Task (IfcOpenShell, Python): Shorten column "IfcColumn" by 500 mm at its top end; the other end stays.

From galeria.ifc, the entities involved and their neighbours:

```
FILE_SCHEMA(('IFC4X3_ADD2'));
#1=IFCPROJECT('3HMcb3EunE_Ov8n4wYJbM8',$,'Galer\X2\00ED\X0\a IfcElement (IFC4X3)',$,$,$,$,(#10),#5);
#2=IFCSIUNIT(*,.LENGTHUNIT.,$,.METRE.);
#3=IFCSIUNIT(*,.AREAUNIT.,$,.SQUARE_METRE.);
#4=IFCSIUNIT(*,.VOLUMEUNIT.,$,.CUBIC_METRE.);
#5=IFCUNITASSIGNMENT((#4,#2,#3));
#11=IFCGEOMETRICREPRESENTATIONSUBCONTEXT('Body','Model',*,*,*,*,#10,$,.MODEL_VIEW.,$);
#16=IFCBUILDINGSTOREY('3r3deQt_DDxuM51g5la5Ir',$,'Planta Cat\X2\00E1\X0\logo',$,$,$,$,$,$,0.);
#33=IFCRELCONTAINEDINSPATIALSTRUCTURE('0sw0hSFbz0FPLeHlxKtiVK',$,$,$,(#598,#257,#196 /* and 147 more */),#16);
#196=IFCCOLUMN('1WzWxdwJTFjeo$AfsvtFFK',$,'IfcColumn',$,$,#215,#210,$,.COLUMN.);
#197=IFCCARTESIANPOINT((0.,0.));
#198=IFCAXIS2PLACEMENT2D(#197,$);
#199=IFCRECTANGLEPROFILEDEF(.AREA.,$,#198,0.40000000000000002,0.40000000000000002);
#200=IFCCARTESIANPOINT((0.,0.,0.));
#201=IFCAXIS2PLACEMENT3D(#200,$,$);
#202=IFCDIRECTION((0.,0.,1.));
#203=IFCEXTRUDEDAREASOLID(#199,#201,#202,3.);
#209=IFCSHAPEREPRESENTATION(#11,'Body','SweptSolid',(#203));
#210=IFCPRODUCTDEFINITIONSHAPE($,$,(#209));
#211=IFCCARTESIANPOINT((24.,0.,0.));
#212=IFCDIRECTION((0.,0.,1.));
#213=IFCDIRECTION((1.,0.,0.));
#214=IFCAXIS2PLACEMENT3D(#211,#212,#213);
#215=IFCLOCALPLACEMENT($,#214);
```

```python
import ifcopenshell
import ifcopenshell.util.representation
import ifcopenshell.util.unit

model = ifcopenshell.open("galeria.ifc")
unit_scale = ifcopenshell.util.unit.calculate_unit_scale(model)

member = model.by_id(196)
change = -0.5 / unit_scale

# The extrusion runs towards the end named, so only its depth changes.
body = ifcopenshell.util.representation.get_representation(member, "Model", "Body")
solid = body.Items[0]
old_length = solid.Depth
solid.Depth += change

print(f"length {old_length:g} -> {solid.Depth:g}")

model.write("galeria-out.ifc")
```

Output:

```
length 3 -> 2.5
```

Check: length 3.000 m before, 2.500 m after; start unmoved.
